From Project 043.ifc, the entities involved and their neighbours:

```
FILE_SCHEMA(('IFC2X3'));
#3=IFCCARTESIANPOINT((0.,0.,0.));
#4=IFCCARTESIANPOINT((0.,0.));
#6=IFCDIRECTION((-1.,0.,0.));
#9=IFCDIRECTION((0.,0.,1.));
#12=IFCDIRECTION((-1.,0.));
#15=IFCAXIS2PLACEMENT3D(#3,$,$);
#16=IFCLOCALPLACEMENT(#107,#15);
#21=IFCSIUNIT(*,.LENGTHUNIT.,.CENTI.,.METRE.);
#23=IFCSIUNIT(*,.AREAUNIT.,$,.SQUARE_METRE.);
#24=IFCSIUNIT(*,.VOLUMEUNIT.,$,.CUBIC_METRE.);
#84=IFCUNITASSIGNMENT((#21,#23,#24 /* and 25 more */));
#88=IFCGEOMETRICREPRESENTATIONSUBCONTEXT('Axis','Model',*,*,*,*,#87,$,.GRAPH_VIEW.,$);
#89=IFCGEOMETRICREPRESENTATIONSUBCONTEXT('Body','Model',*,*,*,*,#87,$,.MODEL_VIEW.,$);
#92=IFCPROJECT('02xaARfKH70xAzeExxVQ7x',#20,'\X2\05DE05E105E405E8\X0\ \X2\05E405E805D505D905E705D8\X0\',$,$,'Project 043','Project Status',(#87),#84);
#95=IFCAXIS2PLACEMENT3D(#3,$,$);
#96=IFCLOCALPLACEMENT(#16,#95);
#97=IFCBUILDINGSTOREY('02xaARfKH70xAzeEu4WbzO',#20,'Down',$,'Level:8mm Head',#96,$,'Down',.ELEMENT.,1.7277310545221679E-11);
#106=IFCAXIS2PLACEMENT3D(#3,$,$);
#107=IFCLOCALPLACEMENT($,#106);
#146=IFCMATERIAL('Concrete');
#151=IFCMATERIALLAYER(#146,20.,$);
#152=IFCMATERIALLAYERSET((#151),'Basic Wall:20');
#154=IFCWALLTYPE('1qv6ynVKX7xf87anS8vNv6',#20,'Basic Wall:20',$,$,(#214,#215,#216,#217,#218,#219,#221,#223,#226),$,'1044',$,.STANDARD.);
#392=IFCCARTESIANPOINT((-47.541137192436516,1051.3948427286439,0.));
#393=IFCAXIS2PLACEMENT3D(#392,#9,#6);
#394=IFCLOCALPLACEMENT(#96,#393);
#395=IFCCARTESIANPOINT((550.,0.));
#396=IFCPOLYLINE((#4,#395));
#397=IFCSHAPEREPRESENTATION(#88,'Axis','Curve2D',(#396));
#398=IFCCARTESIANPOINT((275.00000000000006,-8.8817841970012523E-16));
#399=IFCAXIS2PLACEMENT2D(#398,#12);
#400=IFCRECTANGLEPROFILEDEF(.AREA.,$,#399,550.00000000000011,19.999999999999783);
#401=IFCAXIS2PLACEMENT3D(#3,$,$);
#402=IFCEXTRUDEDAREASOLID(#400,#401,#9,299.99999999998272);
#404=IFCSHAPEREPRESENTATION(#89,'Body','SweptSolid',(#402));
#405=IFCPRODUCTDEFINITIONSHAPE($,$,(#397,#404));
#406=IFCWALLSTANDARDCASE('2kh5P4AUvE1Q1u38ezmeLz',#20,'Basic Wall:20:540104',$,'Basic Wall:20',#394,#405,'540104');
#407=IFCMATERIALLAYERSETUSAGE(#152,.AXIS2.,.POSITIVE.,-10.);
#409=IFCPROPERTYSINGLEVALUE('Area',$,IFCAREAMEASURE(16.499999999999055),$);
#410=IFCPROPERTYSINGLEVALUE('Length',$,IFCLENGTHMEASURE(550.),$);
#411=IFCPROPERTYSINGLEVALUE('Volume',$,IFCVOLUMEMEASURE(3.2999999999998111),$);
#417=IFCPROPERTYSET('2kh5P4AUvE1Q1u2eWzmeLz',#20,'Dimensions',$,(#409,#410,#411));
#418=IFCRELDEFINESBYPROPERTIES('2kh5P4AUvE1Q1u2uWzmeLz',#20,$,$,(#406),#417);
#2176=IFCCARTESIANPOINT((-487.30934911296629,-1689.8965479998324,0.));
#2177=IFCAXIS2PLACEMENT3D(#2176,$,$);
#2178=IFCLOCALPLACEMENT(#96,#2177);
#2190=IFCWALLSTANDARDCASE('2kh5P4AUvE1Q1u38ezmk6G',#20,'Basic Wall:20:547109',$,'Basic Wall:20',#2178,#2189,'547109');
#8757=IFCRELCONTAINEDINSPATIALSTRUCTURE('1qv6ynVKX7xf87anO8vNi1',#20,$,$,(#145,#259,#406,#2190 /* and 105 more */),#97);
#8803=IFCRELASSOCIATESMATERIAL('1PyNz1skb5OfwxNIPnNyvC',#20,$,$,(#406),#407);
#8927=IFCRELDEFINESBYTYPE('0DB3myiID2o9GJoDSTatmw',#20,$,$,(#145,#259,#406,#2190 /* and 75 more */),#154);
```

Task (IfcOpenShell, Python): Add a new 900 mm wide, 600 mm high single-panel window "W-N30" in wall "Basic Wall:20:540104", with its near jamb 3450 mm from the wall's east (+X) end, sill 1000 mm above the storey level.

```python
import numpy as np
import ifcopenshell
import ifcopenshell.api.feature
import ifcopenshell.api.geometry
import ifcopenshell.api.pset
import ifcopenshell.api.root
import ifcopenshell.api.spatial
import ifcopenshell.api.type
import ifcopenshell.geom
import ifcopenshell.util.element
import ifcopenshell.util.placement
import ifcopenshell.util.representation
import ifcopenshell.util.shape
import ifcopenshell.util.unit

model = ifcopenshell.open("Project 043.ifc")
unit_scale = ifcopenshell.util.unit.calculate_unit_scale(model)
area_scale = ifcopenshell.util.unit.calculate_unit_scale(model, "AREAUNIT")
volume_scale = ifcopenshell.util.unit.calculate_unit_scale(model, "VOLUMEUNIT")
settings = ifcopenshell.geom.settings()


def volume(element):
    """Net volume in cubic metres, openings subtracted."""
    shape = ifcopenshell.geom.create_shape(settings, element)
    return ifcopenshell.util.shape.get_volume(shape.geometry)


wall = model.by_guid("2kh5P4AUvE1Q1u38ezmeLz")
storey = ifcopenshell.util.element.get_container(wall, ifc_class="IfcBuildingStorey")
context = ifcopenshell.util.representation.get_context(model, "Model", "Body", "MODEL_VIEW")
before = volume(wall)

width, height, from_end, sill = 0.9, 0.6, 3.45, 1  # metres

# The wall runs along its own X axis, and the end named is its -X end.
wall_shape = ifcopenshell.geom.create_shape(settings, wall)
x, y, z = ifcopenshell.util.shape.get_vertices(wall_shape.geometry).T
start = x.min() + from_end
face, thickness = float(y.min()), float(y.max() - y.min())
wall_matrix = ifcopenshell.util.placement.get_local_placement(wall.ObjectPlacement)
level = ifcopenshell.util.placement.get_local_placement(storey.ObjectPlacement)[2, 3]


def in_wall(x, y):
    """Placement at x, y metres in the wall's axes, at sill height."""
    matrix = wall_matrix.copy()
    matrix[:, 3] = wall_matrix @ np.array([x / unit_scale, y / unit_scale, 0.0, 1.0])
    matrix[2, 3] = level + sill / unit_scale
    return matrix


# Opening: a box that overshoots both wall faces by 50 mm.
opening = ifcopenshell.api.root.create_entity(model, ifc_class="IfcOpeningElement")
box = ifcopenshell.api.geometry.add_wall_representation(
    model, context=context, length=width, height=height, thickness=thickness + 0.1
)
ifcopenshell.api.geometry.assign_representation(model, product=opening, representation=box)
ifcopenshell.api.geometry.edit_object_placement(model, product=opening, matrix=in_wall(start, face - 0.05), is_si=False)
ifcopenshell.api.feature.add_feature(model, feature=opening, element=wall)

window = ifcopenshell.api.root.create_entity(model, ifc_class="IfcWindow", name="W-N30")
window.OverallWidth, window.OverallHeight = width / unit_scale, height / unit_scale
body = ifcopenshell.api.geometry.add_window_representation(
    model,
    context=context,
    overall_width=window.OverallWidth,
    overall_height=window.OverallHeight,
    partition_type="SINGLE_PANEL",
)
ifcopenshell.api.geometry.assign_representation(model, product=window, representation=body)
ifcopenshell.api.spatial.assign_container(model, products=[window], relating_structure=storey)
fills = ifcopenshell.api.feature.add_filling(model, opening=opening, element=window)
fills.OwnerHistory = window.OwnerHistory  # required in IFC2X3

# IFC2X3 keeps the operation on the window style.
style = ifcopenshell.api.root.create_entity(model, ifc_class="IfcWindowStyle", name="W-N30")
style.OperationType, style.ConstructionType = "SINGLE_PANEL", "NOTDEFINED"
style.ParameterTakesPrecedence = style.Sizeable = False
ifcopenshell.api.type.assign_type(model, related_objects=[window], relating_type=style)

# Centre the window in the wall's thickness.
ifcopenshell.api.geometry.edit_object_placement(model, product=window, matrix=in_wall(start, face), is_si=False)
window_shape = ifcopenshell.geom.create_shape(settings, window)
depth = ifcopenshell.util.shape.get_vertices(window_shape.geometry)[:, 1]
offset = face + thickness / 2 - (depth.min() + depth.max()) / 2
ifcopenshell.api.geometry.edit_object_placement(model, product=window, matrix=in_wall(start, offset), is_si=False)

after = volume(wall)

# Update the wall's stored quantities.
pset = model.by_id(ifcopenshell.util.element.get_pset(wall, "Dimensions", should_inherit=False)["id"])
ifcopenshell.api.pset.edit_pset(model, pset=pset, properties={
    "Area": model.create_entity("IfcAreaMeasure", after / thickness / area_scale),
    "Volume": model.create_entity("IfcVolumeMeasure", after / volume_scale),
})

print(f"wall volume {before:.3f} -> {after:.3f} m3")

model.write("Project 043_edited.ifc")
```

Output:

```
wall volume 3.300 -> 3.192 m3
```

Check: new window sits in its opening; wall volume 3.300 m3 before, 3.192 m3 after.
